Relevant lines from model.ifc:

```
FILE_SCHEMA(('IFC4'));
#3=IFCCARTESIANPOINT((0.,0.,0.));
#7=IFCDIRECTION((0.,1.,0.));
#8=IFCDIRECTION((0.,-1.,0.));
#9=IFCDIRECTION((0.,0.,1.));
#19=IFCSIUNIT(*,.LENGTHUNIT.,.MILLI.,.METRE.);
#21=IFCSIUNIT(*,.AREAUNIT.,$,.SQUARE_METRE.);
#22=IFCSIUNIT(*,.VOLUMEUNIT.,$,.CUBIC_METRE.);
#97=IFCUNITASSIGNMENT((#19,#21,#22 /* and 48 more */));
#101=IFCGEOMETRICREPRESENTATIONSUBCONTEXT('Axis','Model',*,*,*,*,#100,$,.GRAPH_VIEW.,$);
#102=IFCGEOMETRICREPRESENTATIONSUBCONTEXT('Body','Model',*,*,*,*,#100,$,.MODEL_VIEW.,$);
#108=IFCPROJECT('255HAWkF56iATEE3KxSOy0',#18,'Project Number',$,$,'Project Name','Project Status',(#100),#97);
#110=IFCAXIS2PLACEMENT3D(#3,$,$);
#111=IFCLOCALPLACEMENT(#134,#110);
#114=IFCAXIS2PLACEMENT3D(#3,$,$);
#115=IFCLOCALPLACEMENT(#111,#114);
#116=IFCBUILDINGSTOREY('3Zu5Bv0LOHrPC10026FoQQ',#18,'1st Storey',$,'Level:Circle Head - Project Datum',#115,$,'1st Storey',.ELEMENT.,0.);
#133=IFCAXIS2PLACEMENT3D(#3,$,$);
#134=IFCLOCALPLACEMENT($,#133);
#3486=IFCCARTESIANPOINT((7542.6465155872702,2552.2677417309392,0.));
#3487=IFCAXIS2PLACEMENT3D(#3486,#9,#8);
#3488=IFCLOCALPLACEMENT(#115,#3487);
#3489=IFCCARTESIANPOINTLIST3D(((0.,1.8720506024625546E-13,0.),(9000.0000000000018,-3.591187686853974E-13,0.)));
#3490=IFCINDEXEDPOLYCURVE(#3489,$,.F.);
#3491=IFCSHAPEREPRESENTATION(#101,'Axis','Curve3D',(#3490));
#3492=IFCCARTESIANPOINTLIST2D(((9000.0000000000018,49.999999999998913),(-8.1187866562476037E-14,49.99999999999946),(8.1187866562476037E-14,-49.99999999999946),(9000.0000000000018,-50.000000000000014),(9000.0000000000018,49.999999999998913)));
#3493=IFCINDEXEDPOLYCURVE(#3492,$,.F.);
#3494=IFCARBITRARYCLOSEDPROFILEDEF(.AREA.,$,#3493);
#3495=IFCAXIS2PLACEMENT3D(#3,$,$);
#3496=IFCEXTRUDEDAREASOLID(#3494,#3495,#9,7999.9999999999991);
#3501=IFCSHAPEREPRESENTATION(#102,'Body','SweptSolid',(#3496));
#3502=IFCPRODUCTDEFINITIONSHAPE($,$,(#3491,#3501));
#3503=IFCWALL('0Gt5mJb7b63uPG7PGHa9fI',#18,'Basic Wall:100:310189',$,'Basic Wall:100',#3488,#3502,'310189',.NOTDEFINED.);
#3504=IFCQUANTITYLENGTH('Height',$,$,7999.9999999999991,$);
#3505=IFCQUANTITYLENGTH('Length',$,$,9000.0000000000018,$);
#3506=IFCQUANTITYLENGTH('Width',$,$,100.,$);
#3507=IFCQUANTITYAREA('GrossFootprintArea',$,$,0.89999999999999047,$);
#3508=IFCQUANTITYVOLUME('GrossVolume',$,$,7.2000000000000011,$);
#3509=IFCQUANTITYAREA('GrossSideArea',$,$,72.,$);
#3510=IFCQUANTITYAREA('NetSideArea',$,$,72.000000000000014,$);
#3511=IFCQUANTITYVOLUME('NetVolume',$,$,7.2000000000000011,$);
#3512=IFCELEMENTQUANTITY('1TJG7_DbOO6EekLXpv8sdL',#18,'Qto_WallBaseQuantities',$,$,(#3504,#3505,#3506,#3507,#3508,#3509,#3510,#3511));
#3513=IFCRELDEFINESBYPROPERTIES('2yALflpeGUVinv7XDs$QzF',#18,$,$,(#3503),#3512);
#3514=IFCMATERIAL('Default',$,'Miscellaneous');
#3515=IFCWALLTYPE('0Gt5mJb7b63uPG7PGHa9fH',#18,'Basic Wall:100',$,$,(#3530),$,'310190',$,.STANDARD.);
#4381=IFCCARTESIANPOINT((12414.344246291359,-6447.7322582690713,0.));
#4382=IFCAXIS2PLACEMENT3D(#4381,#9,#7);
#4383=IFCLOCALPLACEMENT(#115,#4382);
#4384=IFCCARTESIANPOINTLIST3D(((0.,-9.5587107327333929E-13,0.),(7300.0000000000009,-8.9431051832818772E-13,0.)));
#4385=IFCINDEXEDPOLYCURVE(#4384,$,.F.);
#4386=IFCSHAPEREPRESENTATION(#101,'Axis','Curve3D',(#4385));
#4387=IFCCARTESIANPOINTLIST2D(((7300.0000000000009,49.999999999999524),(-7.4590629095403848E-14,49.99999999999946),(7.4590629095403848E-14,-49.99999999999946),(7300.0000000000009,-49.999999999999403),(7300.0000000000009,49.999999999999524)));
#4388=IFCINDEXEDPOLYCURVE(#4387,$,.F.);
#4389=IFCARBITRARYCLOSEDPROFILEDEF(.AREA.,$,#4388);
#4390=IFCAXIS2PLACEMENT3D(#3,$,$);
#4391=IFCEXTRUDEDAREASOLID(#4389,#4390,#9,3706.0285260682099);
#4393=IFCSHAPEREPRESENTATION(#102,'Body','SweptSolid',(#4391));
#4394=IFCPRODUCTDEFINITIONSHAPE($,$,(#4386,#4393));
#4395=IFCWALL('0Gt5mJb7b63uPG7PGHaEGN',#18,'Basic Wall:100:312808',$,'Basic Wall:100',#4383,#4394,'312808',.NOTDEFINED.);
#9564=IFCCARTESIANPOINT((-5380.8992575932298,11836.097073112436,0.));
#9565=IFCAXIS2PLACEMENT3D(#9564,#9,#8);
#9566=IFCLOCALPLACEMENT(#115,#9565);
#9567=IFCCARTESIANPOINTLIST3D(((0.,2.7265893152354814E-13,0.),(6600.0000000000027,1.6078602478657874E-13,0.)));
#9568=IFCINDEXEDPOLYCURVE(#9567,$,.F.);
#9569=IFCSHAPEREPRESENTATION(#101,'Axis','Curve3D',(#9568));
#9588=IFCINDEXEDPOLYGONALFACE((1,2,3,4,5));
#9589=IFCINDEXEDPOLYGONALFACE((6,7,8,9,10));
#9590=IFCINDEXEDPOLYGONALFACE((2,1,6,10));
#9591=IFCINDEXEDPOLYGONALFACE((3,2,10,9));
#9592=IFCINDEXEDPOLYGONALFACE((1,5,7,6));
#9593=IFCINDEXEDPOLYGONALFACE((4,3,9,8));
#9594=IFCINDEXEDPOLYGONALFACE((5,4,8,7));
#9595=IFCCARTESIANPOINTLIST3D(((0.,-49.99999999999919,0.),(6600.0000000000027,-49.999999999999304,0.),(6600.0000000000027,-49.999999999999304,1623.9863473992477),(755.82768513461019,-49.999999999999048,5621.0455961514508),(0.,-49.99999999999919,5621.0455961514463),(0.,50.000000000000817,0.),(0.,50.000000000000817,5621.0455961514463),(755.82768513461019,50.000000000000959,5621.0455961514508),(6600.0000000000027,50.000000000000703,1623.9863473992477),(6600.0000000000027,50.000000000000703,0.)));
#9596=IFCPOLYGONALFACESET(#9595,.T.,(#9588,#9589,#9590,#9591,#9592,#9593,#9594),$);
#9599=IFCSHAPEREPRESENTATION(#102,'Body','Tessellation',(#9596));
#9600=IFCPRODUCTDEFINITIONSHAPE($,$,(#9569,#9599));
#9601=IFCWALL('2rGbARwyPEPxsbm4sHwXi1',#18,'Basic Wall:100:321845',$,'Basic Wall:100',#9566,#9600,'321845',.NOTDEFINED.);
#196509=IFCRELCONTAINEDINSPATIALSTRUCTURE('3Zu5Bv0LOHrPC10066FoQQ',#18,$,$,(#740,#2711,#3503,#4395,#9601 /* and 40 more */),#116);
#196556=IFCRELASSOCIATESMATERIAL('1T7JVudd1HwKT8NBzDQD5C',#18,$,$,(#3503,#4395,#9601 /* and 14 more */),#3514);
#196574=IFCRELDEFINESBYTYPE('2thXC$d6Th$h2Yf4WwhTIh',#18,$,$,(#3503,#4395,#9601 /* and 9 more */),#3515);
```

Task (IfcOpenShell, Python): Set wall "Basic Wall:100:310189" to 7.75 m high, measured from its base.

```python
import ifcopenshell
import ifcopenshell.api.pset
import ifcopenshell.geom
import ifcopenshell.util.element
import ifcopenshell.util.representation
import ifcopenshell.util.shape
import ifcopenshell.util.unit

model = ifcopenshell.open("model.ifc")
unit_scale = ifcopenshell.util.unit.calculate_unit_scale(model)
area_scale = ifcopenshell.util.unit.calculate_unit_scale(model, "AREAUNIT")
volume_scale = ifcopenshell.util.unit.calculate_unit_scale(model, "VOLUMEUNIT")
settings = ifcopenshell.geom.settings()


def volume(element):
    """Net volume in cubic metres, openings subtracted."""
    shape = ifcopenshell.geom.create_shape(settings, element)
    return ifcopenshell.util.shape.get_volume(shape.geometry)


wall = model.by_guid("0Gt5mJb7b63uPG7PGHa9fI")
before = volume(wall)

body = ifcopenshell.util.representation.get_representation(wall, "Model", "Body")
solid = body.Items[0]
old_height = solid.Depth
solid.Depth = 7750.0
after = volume(wall)
thickness = 0.1  # wall thickness in metres

# Update the stored height, areas and volumes.
qto = model.by_id(ifcopenshell.util.element.get_pset(wall, "Qto_WallBaseQuantities", should_inherit=False)["id"])
ifcopenshell.api.pset.edit_qto(model, qto=qto, properties={
    "Height": solid.Depth,
    "GrossVolume": ifcopenshell.util.element.get_pset(wall, "Qto_WallBaseQuantities", "GrossVolume") * solid.Depth / old_height,
    "GrossSideArea": ifcopenshell.util.element.get_pset(wall, "Qto_WallBaseQuantities", "GrossSideArea") * solid.Depth / old_height,
    "NetSideArea": after / thickness / area_scale,
    "NetVolume": after / volume_scale,
})

print(f"height {old_height:g} -> {solid.Depth:g}, volume {before:.3f} -> {after:.3f} m3")

model.write("model_rev.ifc")
```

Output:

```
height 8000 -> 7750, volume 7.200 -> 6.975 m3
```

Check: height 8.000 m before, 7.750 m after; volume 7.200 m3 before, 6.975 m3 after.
